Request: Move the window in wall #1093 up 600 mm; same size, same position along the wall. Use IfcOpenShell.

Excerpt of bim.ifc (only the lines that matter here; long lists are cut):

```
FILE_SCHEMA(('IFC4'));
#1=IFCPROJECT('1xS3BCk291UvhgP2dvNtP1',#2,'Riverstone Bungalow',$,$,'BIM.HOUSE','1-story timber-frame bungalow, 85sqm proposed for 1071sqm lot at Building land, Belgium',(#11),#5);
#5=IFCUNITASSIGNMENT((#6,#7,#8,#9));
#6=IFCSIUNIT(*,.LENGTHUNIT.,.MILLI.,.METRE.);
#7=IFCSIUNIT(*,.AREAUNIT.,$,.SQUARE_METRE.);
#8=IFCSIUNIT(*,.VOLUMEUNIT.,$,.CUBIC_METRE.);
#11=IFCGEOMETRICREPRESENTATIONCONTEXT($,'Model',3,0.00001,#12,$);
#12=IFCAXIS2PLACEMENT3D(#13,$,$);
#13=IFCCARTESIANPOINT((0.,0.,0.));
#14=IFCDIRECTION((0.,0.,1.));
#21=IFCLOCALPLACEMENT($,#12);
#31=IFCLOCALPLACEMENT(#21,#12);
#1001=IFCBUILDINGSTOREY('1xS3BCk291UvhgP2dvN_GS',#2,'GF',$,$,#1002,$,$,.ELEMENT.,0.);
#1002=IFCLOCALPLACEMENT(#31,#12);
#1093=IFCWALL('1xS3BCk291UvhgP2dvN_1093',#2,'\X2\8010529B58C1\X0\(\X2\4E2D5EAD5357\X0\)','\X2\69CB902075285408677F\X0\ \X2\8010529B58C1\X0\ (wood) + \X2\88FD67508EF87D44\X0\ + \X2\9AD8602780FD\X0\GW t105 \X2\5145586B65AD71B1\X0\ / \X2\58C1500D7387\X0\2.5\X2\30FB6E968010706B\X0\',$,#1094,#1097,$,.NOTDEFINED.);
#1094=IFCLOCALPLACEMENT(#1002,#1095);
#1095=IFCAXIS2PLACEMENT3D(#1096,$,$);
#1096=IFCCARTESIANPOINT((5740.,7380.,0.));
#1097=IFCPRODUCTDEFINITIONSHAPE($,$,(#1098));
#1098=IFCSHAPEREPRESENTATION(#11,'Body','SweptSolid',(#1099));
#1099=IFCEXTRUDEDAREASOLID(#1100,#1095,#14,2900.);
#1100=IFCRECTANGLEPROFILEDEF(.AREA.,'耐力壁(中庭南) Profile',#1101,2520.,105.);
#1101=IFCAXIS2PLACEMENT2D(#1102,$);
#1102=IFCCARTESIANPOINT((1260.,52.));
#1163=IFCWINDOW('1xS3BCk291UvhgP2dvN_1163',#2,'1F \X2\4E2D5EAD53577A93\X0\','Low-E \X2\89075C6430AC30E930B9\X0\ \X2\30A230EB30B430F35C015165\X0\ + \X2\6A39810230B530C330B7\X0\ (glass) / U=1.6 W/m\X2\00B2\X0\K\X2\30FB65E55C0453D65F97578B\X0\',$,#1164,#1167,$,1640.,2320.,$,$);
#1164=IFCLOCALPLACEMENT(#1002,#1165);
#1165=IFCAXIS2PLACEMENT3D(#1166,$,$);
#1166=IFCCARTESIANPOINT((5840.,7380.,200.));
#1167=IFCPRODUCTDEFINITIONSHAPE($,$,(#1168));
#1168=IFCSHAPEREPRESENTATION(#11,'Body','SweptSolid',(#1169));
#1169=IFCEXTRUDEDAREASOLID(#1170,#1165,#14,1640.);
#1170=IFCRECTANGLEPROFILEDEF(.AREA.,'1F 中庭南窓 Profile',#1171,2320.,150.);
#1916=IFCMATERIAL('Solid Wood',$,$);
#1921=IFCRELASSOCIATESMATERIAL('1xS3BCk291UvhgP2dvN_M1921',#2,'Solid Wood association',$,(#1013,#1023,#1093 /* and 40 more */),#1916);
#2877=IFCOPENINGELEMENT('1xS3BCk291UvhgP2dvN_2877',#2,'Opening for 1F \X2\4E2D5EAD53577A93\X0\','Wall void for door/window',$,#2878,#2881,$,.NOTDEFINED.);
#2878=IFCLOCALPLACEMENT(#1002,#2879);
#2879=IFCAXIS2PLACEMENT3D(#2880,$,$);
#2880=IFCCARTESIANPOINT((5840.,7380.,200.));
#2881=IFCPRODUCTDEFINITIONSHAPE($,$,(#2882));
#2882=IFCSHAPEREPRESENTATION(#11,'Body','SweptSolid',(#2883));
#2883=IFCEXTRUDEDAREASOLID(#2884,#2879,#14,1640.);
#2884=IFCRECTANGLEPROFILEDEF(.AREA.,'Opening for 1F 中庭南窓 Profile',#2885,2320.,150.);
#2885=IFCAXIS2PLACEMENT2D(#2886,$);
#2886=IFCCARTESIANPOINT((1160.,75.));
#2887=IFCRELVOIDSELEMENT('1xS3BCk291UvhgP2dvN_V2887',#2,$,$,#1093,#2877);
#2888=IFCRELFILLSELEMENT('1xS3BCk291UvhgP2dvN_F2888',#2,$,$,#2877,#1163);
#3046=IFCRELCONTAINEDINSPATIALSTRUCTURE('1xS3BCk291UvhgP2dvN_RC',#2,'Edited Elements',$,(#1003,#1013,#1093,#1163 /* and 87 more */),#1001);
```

```python
import numpy as np
import ifcopenshell
import ifcopenshell.api.geometry
import ifcopenshell.util.placement
import ifcopenshell.util.unit

model = ifcopenshell.open("bim.ifc")
unit_scale = ifcopenshell.util.unit.calculate_unit_scale(model)

window = model.by_id(1163)
opening = window.FillsVoids[0].RelatingOpeningElement
dz = 600.0

shift = np.array([0.0, 0.0, dz])
# The window is not placed relative to its opening, so move both.
for product in (opening, window):
    matrix = ifcopenshell.util.placement.get_local_placement(product.ObjectPlacement)
    matrix[:3, 3] += shift
    ifcopenshell.api.geometry.edit_object_placement(model, product=product, matrix=matrix, is_si=False)

print(f"moved by {dz * unit_scale:+.3f} m")

model.write("bim_rev.ifc")
```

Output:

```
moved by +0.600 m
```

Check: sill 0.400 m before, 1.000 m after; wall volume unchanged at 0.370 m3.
